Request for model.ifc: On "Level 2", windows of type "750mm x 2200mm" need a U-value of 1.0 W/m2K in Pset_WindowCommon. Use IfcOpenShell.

First a look at what the model holds.

```python
import ifcopenshell
import ifcopenshell.util.element

model = ifcopenshell.open("model.ifc")
print(model.schema)
storey = next(s for s in model.by_type("IfcBuildingStorey") if s.Name == "Level 2")
windows = [e for e in ifcopenshell.util.element.get_decomposition(storey) if e.is_a("IfcWindow")]
seen = {}
for e in windows:
    element_type = ifcopenshell.util.element.get_type(e)
    key = (element_type.Name if element_type != e and element_type else None, ifcopenshell.util.element.get_pset(e, "Pset_WindowCommon", "ThermalTransmittance"))
    seen[key] = seen.get(key, 0) + 1
for (name, value), count in sorted(seen.items(), key=str):
    print(count, "x", name, "|", value)
```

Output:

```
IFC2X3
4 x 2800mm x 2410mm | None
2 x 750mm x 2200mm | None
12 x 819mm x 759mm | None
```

```python
import ifcopenshell
import ifcopenshell.api.pset
import ifcopenshell.util.element

model = ifcopenshell.open("model.ifc")

storey = next(s for s in model.by_type("IfcBuildingStorey") if s.Name == "Level 2")
windows = [e for e in ifcopenshell.util.element.get_decomposition(storey) if e.is_a("IfcWindow")]

count = 0
for e in windows:
    element_type = ifcopenshell.util.element.get_type(e)
    if element_type in (None, e) or element_type.Name != "750mm x 2200mm":
        continue
    # add_pset returns the element's existing set when there is one.
    pset = ifcopenshell.api.pset.add_pset(model, product=e, name="Pset_WindowCommon")
    ifcopenshell.api.pset.edit_pset(model, pset=pset, properties={"ThermalTransmittance": 1.0})
    count += 1

print(count, "windows updated")

model.write("model_edited.ifc")
```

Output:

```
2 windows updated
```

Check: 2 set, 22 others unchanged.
